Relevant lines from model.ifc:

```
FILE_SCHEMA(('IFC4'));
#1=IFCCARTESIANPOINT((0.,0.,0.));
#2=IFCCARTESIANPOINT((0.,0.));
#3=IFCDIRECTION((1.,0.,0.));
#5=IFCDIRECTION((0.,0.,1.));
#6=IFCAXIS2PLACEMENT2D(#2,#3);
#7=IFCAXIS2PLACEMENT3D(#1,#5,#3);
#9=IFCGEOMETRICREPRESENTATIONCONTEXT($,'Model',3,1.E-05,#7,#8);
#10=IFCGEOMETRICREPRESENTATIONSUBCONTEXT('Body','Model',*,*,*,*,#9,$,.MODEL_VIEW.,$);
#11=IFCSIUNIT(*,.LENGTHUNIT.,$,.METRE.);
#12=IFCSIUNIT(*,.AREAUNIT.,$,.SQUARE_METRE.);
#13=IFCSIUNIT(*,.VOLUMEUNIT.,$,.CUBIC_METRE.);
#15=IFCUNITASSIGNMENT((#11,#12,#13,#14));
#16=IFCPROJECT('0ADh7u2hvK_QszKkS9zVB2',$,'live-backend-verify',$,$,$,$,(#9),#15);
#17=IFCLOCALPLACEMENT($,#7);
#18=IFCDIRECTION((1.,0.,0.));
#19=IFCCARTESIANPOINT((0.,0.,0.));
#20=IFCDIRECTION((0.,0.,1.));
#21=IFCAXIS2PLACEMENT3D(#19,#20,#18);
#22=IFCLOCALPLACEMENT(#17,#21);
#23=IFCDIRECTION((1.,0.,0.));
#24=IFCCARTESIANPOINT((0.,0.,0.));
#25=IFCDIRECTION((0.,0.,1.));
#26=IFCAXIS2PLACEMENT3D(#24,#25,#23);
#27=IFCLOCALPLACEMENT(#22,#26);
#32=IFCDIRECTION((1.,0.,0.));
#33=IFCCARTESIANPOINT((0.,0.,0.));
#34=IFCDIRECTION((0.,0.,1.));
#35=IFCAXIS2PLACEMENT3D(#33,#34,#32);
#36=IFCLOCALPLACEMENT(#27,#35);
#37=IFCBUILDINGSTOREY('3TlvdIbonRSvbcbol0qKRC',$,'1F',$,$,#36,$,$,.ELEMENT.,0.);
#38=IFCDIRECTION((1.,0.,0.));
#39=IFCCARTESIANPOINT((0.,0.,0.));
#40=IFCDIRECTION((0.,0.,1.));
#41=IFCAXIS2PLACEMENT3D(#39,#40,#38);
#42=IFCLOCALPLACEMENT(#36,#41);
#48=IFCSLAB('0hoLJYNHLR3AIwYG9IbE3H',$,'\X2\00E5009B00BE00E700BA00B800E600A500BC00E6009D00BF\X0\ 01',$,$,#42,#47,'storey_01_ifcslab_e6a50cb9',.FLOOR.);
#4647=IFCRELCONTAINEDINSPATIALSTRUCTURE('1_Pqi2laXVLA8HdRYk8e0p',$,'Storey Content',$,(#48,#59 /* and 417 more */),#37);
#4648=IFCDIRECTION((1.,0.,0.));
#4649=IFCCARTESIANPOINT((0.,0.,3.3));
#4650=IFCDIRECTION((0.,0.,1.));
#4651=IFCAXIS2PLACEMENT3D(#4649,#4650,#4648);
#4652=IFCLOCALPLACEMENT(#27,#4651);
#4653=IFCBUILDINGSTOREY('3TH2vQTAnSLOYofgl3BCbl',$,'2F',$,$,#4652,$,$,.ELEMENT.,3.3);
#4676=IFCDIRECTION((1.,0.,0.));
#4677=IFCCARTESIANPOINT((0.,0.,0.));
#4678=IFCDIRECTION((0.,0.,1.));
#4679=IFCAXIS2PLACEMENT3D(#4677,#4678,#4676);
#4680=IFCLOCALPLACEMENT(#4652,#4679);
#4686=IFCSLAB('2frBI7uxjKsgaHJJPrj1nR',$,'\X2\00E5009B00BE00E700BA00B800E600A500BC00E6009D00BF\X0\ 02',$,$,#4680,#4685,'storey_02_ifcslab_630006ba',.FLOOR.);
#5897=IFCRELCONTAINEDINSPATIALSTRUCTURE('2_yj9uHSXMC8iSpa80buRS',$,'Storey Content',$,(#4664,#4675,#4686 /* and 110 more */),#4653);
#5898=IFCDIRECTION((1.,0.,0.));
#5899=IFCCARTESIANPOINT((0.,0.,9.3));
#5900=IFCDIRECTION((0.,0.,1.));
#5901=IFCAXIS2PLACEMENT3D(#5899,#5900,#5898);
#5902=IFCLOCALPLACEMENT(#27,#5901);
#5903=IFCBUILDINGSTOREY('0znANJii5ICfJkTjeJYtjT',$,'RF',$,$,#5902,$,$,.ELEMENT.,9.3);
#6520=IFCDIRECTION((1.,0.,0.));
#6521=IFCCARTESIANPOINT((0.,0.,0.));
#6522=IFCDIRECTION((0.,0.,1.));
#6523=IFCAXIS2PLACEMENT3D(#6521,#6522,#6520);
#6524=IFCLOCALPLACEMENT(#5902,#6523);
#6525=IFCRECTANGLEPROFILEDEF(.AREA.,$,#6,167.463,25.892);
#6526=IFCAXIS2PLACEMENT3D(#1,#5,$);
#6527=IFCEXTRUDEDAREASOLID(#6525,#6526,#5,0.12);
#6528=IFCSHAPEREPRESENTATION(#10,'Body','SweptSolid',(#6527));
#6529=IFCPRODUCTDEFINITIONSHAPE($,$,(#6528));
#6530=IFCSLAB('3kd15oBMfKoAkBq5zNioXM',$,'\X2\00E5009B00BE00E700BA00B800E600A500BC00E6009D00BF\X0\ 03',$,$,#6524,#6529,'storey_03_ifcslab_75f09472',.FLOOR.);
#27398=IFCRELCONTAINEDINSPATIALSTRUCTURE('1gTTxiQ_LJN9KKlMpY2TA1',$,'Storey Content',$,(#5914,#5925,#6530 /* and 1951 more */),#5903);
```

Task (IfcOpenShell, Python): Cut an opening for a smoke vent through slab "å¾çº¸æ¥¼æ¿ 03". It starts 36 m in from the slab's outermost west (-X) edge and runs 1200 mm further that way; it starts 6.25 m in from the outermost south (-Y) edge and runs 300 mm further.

```python
import numpy as np
import ifcopenshell
import ifcopenshell.api.feature
import ifcopenshell.api.geometry
import ifcopenshell.api.root
import ifcopenshell.geom
import ifcopenshell.util.placement
import ifcopenshell.util.representation
import ifcopenshell.util.shape
import ifcopenshell.util.unit

model = ifcopenshell.open("model.ifc")
unit_scale = ifcopenshell.util.unit.calculate_unit_scale(model)
settings = ifcopenshell.geom.settings()


def volume(element):
    """Net volume in cubic metres, openings subtracted."""
    shape = ifcopenshell.geom.create_shape(settings, element)
    return ifcopenshell.util.shape.get_volume(shape.geometry)


slab = model.by_guid("3kd15oBMfKoAkBq5zNioXM")
before = volume(slab)

# Extent in the slab's own axes, in metres. The edges named are its -X and -Y sides.
slab_shape = ifcopenshell.geom.create_shape(settings, slab)
vertices = ifcopenshell.util.shape.get_vertices(slab_shape.geometry)
x_min, y_min, bottom = vertices.min(axis=0)
top = vertices[:, 2].max()

opening = ifcopenshell.api.root.create_entity(model, ifc_class="IfcOpeningElement", name="Smoke vent opening", predefined_type="OPENING")
context = ifcopenshell.util.representation.get_context(model, "Model", "Body", "MODEL_VIEW")
width, depth = 1.2, 0.3
outline = [(0.0, 0.0), (width, 0.0), (width, depth), (0.0, depth), (0.0, 0.0)]
# Overshoot both faces by 50 mm so the cut is clean.
shape = ifcopenshell.api.geometry.add_slab_representation(
    model, context=context, depth=top - bottom + 0.1, polyline=outline
)
ifcopenshell.api.geometry.assign_representation(model, product=opening, representation=shape)

matrix = ifcopenshell.util.placement.get_local_placement(slab.ObjectPlacement)
matrix[:, 3] = matrix @ np.append(np.array([x_min + 36, y_min + 6.25, bottom - 0.05]) / unit_scale, 1.0)
ifcopenshell.api.geometry.edit_object_placement(model, product=opening, matrix=matrix, is_si=False)
ifcopenshell.api.feature.add_feature(model, feature=opening, element=slab)

after = volume(slab)

print(f"slab volume {before:.3f} -> {after:.3f} m3")

model.write("model_updated.ifc")
```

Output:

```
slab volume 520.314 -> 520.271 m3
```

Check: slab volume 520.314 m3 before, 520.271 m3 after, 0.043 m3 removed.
